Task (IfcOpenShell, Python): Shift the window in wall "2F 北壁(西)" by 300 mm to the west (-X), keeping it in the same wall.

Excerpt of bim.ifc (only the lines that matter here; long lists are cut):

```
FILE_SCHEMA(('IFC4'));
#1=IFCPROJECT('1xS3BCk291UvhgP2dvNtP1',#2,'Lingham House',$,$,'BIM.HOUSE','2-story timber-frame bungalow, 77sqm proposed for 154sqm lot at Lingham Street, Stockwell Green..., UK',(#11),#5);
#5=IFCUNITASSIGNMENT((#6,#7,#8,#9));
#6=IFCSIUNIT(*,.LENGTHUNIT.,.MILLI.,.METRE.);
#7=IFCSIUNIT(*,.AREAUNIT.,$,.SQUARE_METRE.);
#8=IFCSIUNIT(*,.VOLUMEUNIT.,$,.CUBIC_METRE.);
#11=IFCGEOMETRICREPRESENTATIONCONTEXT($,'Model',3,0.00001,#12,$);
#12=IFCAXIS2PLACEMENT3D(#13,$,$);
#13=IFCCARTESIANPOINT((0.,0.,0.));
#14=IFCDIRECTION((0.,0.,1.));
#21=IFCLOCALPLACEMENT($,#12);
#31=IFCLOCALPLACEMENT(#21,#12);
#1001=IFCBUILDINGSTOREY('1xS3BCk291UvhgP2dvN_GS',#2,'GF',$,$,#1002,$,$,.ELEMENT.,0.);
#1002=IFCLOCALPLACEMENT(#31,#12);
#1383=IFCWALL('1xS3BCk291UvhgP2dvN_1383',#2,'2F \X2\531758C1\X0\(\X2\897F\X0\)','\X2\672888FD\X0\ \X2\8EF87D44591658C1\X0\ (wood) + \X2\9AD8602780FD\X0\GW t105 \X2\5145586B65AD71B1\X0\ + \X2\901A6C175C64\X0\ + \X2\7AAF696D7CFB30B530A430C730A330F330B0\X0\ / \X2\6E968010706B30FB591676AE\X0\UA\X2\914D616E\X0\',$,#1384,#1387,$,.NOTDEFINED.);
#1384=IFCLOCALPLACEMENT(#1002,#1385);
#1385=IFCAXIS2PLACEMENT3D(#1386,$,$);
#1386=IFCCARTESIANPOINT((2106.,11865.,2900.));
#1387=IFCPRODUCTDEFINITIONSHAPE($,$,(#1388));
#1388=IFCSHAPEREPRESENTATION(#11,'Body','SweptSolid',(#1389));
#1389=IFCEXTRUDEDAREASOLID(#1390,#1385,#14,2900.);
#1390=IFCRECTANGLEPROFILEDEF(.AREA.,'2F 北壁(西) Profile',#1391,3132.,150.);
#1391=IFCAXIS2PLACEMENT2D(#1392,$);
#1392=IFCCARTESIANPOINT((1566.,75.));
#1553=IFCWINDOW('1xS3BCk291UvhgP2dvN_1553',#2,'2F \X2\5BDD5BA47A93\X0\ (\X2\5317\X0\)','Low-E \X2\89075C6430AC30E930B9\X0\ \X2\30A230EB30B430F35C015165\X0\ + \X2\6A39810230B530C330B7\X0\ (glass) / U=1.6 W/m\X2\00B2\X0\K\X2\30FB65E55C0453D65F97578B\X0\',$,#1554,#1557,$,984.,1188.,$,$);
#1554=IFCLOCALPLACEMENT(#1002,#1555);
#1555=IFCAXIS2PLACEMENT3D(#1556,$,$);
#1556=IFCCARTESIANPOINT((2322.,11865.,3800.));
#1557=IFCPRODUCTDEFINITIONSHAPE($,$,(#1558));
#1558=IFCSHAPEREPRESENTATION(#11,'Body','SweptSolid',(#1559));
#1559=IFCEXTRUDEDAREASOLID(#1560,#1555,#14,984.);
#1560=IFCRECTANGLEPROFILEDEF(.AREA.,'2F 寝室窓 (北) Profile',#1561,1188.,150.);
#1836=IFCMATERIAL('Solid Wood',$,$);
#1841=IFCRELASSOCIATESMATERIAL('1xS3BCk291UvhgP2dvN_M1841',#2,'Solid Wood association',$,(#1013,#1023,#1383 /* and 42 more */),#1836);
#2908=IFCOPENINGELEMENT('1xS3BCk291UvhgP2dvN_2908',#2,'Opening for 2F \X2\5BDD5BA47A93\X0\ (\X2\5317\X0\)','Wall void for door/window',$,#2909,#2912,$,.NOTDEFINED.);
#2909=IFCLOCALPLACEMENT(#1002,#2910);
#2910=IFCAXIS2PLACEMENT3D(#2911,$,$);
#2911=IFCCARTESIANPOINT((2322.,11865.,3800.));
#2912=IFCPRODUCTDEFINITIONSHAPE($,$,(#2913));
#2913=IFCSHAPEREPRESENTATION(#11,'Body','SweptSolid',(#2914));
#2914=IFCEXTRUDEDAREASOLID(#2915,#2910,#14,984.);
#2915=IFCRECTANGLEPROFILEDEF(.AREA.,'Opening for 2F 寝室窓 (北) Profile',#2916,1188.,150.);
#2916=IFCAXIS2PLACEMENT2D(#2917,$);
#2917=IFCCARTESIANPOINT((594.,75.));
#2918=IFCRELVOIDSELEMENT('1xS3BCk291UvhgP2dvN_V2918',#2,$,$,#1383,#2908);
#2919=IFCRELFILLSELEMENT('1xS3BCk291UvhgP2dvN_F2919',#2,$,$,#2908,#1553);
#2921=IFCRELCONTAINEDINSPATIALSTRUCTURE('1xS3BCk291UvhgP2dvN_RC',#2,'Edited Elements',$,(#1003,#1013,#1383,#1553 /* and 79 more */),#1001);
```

```python
import ifcopenshell
import ifcopenshell.api.geometry
import ifcopenshell.util.placement
import ifcopenshell.util.unit

model = ifcopenshell.open("bim.ifc")
unit_scale = ifcopenshell.util.unit.calculate_unit_scale(model)

window = model.by_guid("1xS3BCk291UvhgP2dvN_1553")
opening = window.FillsVoids[0].RelatingOpeningElement
wall = opening.VoidsElements[0].RelatingBuildingElement

wall_matrix = ifcopenshell.util.placement.get_local_placement(wall.ObjectPlacement)
shift = wall_matrix[:3, 0] * -0.3 / unit_scale
before = ifcopenshell.util.placement.get_local_placement(window.ObjectPlacement)[:3, 3].copy()

# The window is not placed relative to its opening, so move both.
for product in (opening, window):
    matrix = ifcopenshell.util.placement.get_local_placement(product.ObjectPlacement)
    matrix[:3, 3] += shift
    ifcopenshell.api.geometry.edit_object_placement(model, product=product, matrix=matrix, is_si=False)

after = ifcopenshell.util.placement.get_local_placement(window.ObjectPlacement)[:3, 3]
print("window moved by", (after - before).round(3) + 0.0)

model.write("bim_edited.ifc")
```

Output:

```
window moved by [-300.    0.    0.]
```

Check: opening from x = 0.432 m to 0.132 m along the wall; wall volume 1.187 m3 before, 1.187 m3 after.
